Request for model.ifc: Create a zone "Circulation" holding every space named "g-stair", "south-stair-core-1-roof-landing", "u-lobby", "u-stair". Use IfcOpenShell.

First a look at what the model holds.

```python
import ifcopenshell

model = ifcopenshell.open("model.ifc")
print(model.schema)
seen = {}
for space in model.by_type("IfcSpace"):
    seen[space.LongName] = seen.get(space.LongName, 0) + 1
for name, count in sorted(seen.items(), key=str):
    print(count, "x", name)
print("zones:", [z.Name for z in model.by_type("IfcZone")][:20])
```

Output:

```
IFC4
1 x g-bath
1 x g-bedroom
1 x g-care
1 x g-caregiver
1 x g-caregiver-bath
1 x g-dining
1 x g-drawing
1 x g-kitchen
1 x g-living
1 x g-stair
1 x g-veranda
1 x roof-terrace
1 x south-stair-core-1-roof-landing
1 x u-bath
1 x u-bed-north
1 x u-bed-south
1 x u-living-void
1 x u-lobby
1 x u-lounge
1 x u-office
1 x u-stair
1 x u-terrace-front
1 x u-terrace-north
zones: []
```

```python
import ifcopenshell
import ifcopenshell.api.group
import ifcopenshell.api.root

model = ifcopenshell.open("model.ifc")

names = {"g-stair", "south-stair-core-1-roof-landing", "u-lobby", "u-stair"}
spaces = [s for s in model.by_type("IfcSpace") if s.LongName in names]

zone = ifcopenshell.api.root.create_entity(model, ifc_class="IfcZone", name="Circulation")
ifcopenshell.api.group.assign_group(model, products=spaces, group=zone)
print(len(spaces), "spaces in", zone.Name)

model.write("model-out.ifc")
```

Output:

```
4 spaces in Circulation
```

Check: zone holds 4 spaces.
